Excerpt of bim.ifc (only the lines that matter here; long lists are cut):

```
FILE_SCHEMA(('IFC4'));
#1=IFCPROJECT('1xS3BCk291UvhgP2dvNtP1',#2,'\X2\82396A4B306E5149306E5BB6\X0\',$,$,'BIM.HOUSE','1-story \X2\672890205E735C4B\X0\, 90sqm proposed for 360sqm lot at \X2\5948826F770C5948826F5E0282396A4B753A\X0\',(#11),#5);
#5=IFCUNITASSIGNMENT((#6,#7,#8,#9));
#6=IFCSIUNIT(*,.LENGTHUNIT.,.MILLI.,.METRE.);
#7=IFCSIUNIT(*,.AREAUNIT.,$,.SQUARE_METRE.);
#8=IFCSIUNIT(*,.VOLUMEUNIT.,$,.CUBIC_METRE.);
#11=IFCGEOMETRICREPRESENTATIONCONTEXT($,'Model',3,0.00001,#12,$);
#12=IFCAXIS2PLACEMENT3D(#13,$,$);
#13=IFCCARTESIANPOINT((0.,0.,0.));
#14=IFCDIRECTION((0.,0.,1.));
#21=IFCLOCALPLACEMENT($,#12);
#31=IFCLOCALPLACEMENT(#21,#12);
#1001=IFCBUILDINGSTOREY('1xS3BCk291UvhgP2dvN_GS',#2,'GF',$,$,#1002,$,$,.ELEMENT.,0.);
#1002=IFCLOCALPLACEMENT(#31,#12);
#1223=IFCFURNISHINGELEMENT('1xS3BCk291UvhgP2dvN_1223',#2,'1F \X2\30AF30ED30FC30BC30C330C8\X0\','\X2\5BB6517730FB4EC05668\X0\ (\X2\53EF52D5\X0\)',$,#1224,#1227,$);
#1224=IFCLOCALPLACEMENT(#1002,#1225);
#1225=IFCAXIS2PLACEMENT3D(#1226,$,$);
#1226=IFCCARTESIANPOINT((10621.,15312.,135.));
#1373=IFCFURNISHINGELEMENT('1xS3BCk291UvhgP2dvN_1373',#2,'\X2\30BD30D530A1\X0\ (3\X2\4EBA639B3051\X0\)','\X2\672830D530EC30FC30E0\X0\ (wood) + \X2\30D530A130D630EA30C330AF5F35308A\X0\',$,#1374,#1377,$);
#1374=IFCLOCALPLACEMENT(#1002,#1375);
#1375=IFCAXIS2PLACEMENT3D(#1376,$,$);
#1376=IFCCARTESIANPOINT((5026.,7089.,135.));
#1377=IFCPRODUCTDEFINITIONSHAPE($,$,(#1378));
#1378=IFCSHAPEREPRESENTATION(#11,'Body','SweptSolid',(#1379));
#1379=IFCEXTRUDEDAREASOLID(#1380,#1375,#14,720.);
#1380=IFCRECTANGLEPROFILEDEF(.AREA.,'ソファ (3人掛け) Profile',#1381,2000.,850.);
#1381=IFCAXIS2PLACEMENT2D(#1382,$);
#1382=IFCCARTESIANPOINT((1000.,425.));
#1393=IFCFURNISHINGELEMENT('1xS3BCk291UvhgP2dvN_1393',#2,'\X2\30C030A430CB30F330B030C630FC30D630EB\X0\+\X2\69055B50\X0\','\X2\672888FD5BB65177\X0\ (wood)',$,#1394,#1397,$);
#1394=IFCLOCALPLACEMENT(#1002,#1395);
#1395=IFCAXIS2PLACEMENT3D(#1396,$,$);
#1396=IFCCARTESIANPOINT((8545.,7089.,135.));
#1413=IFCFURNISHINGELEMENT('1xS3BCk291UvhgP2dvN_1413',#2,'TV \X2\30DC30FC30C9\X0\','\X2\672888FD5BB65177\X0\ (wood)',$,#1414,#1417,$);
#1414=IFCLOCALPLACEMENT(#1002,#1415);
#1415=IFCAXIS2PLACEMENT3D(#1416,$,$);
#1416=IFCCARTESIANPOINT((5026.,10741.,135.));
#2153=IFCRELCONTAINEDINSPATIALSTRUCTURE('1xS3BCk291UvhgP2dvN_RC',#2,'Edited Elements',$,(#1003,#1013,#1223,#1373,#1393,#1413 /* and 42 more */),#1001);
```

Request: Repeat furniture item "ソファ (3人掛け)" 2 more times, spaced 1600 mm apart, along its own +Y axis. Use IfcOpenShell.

```python
import ifcopenshell
import ifcopenshell.api.geometry
import ifcopenshell.api.root
import ifcopenshell.util.element
import ifcopenshell.util.placement
import ifcopenshell.util.unit

model = ifcopenshell.open("bim.ifc")
unit_scale = ifcopenshell.util.unit.calculate_unit_scale(model)


def reuse_history(source, copy):
    """copy_class also copies each property set's owner history, people and application; keep the originals."""
    for rel in copy.IsDefinedBy:
        if rel.is_a("IfcRelDefinesByProperties") and (history := rel.RelatingPropertyDefinition.OwnerHistory):
            rel.RelatingPropertyDefinition.OwnerHistory = source.OwnerHistory
            ifcopenshell.util.element.remove_deep2(model, history)


source = model.by_guid("1xS3BCk291UvhgP2dvN_1373")
base = ifcopenshell.util.placement.get_local_placement(source.ObjectPlacement)
step = base[:3, 1] * 1.6 / unit_scale

for i in range(1, 3):
    copy = ifcopenshell.api.root.copy_class(model, product=source)
    copy.Representation = ifcopenshell.util.element.copy_deep(
        model, source.Representation, exclude=["IfcGeometricRepresentationContext", "IfcRepresentationMap"]
    )
    reuse_history(source, copy)
    matrix = base.copy()
    matrix[:3, 3] += i * step
    print("added at", matrix[:3, 3].round(3) + 0.0)
    ifcopenshell.api.geometry.edit_object_placement(model, product=copy, matrix=matrix, is_si=False)

model.write("bim_rev.ifc")
```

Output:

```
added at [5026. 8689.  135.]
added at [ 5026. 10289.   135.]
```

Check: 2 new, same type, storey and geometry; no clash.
